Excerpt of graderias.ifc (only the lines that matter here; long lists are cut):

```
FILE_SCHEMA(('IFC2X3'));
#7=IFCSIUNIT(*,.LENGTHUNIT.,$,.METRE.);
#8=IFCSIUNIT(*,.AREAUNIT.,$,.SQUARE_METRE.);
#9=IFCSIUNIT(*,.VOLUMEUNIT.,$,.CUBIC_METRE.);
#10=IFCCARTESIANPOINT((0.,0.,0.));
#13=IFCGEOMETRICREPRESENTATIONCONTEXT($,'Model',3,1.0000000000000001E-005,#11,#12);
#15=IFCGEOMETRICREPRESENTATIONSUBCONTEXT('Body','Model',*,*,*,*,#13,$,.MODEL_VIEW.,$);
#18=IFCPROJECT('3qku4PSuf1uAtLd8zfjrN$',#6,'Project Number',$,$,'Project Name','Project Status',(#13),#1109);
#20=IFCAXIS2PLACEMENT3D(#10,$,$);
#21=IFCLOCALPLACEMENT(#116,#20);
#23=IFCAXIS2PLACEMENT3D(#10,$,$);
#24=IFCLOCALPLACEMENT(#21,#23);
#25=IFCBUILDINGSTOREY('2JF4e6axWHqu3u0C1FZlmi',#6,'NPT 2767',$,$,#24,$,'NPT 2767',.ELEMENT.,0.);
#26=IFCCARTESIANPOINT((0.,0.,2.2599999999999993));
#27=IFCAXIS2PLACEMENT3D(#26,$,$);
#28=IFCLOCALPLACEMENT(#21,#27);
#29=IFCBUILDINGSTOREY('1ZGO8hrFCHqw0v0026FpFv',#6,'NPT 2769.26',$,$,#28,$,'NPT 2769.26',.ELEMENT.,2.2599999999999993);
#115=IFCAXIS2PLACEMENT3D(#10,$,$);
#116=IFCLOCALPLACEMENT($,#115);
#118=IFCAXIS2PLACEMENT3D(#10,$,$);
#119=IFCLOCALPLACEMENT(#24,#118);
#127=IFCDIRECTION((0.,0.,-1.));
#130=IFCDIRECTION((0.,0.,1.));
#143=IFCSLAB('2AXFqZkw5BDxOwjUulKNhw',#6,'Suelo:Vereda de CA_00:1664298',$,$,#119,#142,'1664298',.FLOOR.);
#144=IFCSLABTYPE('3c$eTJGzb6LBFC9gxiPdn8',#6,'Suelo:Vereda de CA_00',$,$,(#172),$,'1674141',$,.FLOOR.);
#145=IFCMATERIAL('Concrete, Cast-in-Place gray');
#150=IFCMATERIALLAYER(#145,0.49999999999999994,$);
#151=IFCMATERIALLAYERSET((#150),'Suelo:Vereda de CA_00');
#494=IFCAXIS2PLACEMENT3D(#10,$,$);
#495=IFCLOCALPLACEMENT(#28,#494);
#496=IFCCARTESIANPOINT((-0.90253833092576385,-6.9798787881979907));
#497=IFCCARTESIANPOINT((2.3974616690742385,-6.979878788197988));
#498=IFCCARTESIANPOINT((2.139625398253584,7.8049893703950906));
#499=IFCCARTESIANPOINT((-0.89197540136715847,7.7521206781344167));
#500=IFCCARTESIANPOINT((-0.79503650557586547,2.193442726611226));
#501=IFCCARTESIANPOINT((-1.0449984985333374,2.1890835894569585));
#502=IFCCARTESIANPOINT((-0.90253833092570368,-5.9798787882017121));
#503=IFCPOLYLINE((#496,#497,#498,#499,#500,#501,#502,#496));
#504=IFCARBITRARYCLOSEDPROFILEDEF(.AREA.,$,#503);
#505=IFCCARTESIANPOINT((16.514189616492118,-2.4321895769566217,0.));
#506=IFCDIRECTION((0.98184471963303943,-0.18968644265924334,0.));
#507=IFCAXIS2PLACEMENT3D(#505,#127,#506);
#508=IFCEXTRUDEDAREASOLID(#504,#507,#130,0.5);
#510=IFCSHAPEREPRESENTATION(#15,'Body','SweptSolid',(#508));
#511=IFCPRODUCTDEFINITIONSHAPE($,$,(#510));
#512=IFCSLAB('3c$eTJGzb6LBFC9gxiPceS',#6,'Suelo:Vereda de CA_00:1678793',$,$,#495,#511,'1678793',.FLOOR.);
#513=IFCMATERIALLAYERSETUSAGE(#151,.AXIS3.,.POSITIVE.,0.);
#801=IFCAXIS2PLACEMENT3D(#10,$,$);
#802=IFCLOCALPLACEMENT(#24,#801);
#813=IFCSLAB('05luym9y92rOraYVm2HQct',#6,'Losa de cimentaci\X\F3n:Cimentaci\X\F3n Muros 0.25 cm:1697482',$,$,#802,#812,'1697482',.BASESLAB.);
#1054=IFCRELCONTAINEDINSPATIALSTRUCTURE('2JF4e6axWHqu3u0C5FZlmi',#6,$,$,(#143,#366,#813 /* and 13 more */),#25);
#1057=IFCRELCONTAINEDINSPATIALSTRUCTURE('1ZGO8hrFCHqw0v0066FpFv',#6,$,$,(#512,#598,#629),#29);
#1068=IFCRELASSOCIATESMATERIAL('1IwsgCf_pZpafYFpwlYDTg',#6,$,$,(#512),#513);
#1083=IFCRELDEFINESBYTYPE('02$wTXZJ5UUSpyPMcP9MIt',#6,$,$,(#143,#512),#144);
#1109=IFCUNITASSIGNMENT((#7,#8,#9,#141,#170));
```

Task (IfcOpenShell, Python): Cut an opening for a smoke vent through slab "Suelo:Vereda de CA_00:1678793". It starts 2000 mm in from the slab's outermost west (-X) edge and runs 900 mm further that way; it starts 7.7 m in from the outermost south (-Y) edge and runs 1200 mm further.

```python
import numpy as np
import ifcopenshell
import ifcopenshell.api.feature
import ifcopenshell.api.geometry
import ifcopenshell.api.root
import ifcopenshell.geom
import ifcopenshell.util.placement
import ifcopenshell.util.representation
import ifcopenshell.util.shape
import ifcopenshell.util.unit

model = ifcopenshell.open("graderias.ifc")
unit_scale = ifcopenshell.util.unit.calculate_unit_scale(model)
settings = ifcopenshell.geom.settings()


def volume(element):
    """Net volume in cubic metres, openings subtracted."""
    shape = ifcopenshell.geom.create_shape(settings, element)
    return ifcopenshell.util.shape.get_volume(shape.geometry)


slab = model.by_guid("3c$eTJGzb6LBFC9gxiPceS")
before = volume(slab)

# Extent in the slab's own axes, in metres. The edges named are its -X and -Y sides.
slab_shape = ifcopenshell.geom.create_shape(settings, slab)
vertices = ifcopenshell.util.shape.get_vertices(slab_shape.geometry)
x_min, y_min, bottom = vertices.min(axis=0)
top = vertices[:, 2].max()

opening = ifcopenshell.api.root.create_entity(model, ifc_class="IfcOpeningElement", name="Smoke vent opening")
context = ifcopenshell.util.representation.get_context(model, "Model", "Body", "MODEL_VIEW")
width, depth = 0.9, 1.2
outline = [(0.0, 0.0), (width, 0.0), (width, depth), (0.0, depth), (0.0, 0.0)]
# Overshoot both faces by 50 mm so the cut is clean.
shape = ifcopenshell.api.geometry.add_slab_representation(
    model, context=context, depth=top - bottom + 0.1, polyline=outline
)
ifcopenshell.api.geometry.assign_representation(model, product=opening, representation=shape)

matrix = ifcopenshell.util.placement.get_local_placement(slab.ObjectPlacement)
matrix[:, 3] = matrix @ np.append(np.array([x_min + 2, y_min + 7.7, bottom - 0.05]) / unit_scale, 1.0)
ifcopenshell.api.geometry.edit_object_placement(model, product=opening, matrix=matrix, is_si=False)
ifcopenshell.api.feature.add_feature(model, feature=opening, element=slab)

after = volume(slab)

print(f"slab volume {before:.3f} -> {after:.3f} m3")

model.write("graderias_v2.ifc")
```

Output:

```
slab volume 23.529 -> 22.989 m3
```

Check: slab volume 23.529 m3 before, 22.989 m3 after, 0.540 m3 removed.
